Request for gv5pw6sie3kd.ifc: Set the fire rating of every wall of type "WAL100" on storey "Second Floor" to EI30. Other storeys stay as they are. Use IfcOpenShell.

First a look at what the model holds.

```python
import ifcopenshell
import ifcopenshell.util.element

model = ifcopenshell.open("gv5pw6sie3kd.ifc")
print(model.schema)
storey = next(s for s in model.by_type("IfcBuildingStorey") if s.Name == "Second Floor")
walls = [e for e in ifcopenshell.util.element.get_decomposition(storey) if e.is_a("IfcWall")]
seen = {}
for e in walls:
    element_type = ifcopenshell.util.element.get_type(e)
    key = (element_type.Name if element_type != e and element_type else None, ifcopenshell.util.element.get_pset(e, "Pset_WallCommon", "FireRating"))
    seen[key] = seen.get(key, 0) + 1
for (name, value), count in sorted(seen.items(), key=str):
    print(count, "x", name, "|", value)
```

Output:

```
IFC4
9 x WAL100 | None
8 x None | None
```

```python
import ifcopenshell
import ifcopenshell.api.pset
import ifcopenshell.util.element

model = ifcopenshell.open("gv5pw6sie3kd.ifc")

storey = next(s for s in model.by_type("IfcBuildingStorey") if s.Name == "Second Floor")
walls = [e for e in ifcopenshell.util.element.get_decomposition(storey) if e.is_a("IfcWall")]

count = 0
for e in walls:
    element_type = ifcopenshell.util.element.get_type(e)
    if element_type in (None, e) or element_type.Name != "WAL100":
        continue
    # add_pset returns the element's existing set when there is one.
    pset = ifcopenshell.api.pset.add_pset(model, product=e, name="Pset_WallCommon")
    ifcopenshell.api.pset.edit_pset(model, pset=pset, properties={"FireRating": "EI30"})
    count += 1

print(count, "walls updated")

model.write("gv5pw6sie3kd_edited.ifc")
```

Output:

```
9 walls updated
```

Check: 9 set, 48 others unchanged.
